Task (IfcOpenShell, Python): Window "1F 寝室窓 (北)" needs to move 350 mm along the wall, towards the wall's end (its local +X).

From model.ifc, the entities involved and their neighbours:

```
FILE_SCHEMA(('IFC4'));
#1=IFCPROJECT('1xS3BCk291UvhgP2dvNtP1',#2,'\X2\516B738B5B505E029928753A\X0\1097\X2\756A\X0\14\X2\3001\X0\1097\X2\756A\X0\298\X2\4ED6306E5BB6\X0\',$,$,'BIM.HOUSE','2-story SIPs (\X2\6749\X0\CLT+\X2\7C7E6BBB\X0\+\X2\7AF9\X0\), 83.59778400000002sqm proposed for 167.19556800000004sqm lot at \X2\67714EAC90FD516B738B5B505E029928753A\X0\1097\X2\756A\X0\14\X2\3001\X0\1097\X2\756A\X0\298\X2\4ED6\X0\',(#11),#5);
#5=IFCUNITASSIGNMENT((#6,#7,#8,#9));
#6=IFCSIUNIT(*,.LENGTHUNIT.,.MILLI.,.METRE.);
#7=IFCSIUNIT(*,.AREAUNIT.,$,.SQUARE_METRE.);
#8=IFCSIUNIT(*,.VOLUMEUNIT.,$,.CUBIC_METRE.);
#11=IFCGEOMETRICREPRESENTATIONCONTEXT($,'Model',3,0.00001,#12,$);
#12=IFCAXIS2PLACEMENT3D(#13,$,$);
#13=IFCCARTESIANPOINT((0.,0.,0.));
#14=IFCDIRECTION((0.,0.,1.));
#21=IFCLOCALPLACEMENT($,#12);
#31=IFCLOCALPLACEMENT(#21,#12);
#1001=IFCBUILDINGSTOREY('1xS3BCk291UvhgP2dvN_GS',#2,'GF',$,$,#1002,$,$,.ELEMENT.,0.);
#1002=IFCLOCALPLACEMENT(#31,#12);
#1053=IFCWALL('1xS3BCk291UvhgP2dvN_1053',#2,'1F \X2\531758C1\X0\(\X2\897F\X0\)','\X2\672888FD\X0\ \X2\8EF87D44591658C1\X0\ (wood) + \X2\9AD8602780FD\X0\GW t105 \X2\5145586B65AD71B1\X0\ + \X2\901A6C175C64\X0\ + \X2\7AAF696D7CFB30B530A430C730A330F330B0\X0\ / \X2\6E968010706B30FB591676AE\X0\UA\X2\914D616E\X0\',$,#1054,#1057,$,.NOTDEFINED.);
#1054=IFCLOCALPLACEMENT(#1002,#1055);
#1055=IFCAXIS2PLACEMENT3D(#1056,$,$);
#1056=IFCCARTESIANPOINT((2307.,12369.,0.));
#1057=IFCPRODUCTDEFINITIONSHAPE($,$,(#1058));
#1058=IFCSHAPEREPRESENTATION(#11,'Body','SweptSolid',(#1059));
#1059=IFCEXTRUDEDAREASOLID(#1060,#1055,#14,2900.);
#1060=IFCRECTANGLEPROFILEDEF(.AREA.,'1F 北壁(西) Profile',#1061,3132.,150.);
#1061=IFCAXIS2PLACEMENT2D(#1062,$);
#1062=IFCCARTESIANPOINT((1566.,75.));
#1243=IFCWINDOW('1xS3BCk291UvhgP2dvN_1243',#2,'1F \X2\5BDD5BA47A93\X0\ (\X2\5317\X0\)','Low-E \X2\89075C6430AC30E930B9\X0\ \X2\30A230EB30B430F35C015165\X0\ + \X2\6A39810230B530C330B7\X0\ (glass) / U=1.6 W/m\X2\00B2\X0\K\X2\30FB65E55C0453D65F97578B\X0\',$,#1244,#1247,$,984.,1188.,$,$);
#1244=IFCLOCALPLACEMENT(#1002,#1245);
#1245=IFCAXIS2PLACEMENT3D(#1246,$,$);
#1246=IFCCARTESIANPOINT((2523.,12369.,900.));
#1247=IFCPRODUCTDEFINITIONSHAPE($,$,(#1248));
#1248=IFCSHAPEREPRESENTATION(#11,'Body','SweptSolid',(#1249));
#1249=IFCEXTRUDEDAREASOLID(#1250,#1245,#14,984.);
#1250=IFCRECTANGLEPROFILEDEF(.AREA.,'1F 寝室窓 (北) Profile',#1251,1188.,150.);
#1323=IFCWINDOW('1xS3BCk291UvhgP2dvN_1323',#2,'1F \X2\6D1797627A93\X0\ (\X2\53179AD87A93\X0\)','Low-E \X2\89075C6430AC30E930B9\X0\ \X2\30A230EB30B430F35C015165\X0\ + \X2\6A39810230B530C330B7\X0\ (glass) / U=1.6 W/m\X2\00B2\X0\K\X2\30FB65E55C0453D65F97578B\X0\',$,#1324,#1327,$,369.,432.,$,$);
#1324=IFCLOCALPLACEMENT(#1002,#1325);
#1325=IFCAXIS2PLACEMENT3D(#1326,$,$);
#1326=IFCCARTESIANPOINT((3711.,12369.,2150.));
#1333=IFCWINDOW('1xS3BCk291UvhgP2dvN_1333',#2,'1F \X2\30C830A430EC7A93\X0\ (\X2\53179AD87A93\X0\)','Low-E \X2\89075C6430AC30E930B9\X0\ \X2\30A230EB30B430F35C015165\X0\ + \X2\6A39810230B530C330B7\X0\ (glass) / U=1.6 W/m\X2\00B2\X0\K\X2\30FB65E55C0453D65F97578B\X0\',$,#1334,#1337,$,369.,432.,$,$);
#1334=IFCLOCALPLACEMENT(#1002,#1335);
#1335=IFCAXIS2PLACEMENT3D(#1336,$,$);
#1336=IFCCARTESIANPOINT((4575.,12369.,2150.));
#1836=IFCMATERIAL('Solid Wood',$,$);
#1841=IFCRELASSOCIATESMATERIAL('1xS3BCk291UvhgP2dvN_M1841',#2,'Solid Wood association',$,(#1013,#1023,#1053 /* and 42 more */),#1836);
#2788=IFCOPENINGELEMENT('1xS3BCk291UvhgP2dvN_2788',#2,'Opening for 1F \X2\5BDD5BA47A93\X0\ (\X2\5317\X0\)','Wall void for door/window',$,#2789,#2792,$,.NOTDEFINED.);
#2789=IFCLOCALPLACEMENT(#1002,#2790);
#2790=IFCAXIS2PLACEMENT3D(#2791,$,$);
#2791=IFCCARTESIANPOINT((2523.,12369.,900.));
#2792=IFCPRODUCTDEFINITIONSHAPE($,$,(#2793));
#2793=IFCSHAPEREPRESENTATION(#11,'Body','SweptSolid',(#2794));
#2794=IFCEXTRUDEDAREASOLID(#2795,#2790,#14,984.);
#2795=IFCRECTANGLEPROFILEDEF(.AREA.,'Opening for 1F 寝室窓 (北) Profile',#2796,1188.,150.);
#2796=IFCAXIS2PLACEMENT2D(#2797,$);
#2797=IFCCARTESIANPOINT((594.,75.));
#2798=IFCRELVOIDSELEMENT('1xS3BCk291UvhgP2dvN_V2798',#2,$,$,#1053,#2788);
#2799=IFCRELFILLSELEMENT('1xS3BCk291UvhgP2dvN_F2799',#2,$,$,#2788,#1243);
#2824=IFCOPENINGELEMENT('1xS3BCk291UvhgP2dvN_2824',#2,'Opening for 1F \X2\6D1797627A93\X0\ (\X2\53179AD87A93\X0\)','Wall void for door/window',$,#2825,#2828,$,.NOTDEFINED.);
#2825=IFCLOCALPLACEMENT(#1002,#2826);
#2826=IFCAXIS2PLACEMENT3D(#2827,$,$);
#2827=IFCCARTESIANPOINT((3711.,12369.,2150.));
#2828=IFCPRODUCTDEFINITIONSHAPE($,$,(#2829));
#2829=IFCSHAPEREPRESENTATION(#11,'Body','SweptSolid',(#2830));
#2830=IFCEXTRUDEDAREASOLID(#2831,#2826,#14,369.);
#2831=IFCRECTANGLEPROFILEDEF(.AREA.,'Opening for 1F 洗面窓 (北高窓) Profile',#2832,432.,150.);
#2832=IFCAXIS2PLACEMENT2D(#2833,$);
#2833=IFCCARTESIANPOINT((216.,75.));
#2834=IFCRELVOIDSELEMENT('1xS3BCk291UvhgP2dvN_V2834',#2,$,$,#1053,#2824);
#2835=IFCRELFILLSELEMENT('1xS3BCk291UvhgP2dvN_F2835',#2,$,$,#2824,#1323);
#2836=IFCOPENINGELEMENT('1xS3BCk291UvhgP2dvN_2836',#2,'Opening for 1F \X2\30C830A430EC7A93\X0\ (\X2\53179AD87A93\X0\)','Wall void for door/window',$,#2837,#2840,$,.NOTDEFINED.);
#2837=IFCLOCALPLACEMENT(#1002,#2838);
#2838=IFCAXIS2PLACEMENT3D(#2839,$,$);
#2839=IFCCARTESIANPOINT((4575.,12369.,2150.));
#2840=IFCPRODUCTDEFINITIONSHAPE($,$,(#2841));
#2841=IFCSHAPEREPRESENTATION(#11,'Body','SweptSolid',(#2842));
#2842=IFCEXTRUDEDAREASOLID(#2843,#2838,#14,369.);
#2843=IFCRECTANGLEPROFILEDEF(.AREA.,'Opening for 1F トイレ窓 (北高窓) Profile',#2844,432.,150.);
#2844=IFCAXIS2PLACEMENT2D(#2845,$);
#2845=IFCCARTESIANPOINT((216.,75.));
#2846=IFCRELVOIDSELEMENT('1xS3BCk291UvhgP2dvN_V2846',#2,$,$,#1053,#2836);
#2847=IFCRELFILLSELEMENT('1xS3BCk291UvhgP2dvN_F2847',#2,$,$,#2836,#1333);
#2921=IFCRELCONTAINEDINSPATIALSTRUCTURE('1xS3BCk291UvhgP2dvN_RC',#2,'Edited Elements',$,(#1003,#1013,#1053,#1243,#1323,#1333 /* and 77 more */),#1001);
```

```python
import ifcopenshell
import ifcopenshell.api.geometry
import ifcopenshell.util.placement
import ifcopenshell.util.unit

model = ifcopenshell.open("model.ifc")
unit_scale = ifcopenshell.util.unit.calculate_unit_scale(model)

window = model.by_guid("1xS3BCk291UvhgP2dvN_1243")
opening = window.FillsVoids[0].RelatingOpeningElement
wall = opening.VoidsElements[0].RelatingBuildingElement

wall_matrix = ifcopenshell.util.placement.get_local_placement(wall.ObjectPlacement)
shift = wall_matrix[:3, 0] * 0.35 / unit_scale
before = ifcopenshell.util.placement.get_local_placement(window.ObjectPlacement)[:3, 3].copy()

# The window is not placed relative to its opening, so move both.
for product in (opening, window):
    matrix = ifcopenshell.util.placement.get_local_placement(product.ObjectPlacement)
    matrix[:3, 3] += shift
    ifcopenshell.api.geometry.edit_object_placement(model, product=product, matrix=matrix, is_si=False)

after = ifcopenshell.util.placement.get_local_placement(window.ObjectPlacement)[:3, 3]
print("window moved by", (after - before).round(3) + 0.0)

model.write("model_edited.ifc")
```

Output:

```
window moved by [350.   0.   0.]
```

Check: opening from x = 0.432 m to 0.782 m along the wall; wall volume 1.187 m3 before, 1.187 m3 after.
